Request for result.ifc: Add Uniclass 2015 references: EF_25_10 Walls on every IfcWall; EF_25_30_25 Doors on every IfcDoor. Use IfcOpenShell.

First a look at what the model holds.

```python
import ifcopenshell

model = ifcopenshell.open("result.ifc")
print(model.schema)
print("classifications:", [c.Name for c in model.by_type("IfcClassification")])
for ifc_class in ("IfcDoor", "IfcRoof", "IfcStair", "IfcWall", "IfcWindow"):
    print(ifc_class, len(model.by_type(ifc_class)))
```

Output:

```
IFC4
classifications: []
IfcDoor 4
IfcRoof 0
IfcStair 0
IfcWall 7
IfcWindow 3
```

```python
import ifcopenshell
import ifcopenshell.api.classification

model = ifcopenshell.open("result.ifc")

system = ifcopenshell.api.classification.add_classification(model, classification="Uniclass 2015")

codes = {
    "IfcWall": ("EF_25_10", "Walls"),
    "IfcDoor": ("EF_25_30_25", "Doors"),
}
for ifc_class, (code, name) in codes.items():
    products = model.by_type(ifc_class)
    ifcopenshell.api.classification.add_reference(
        model, products=products, classification=system, identification=code, name=name
    )
    print(code, len(products))

model.write("result_edited.ifc")
```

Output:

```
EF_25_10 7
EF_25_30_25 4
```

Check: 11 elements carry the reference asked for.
